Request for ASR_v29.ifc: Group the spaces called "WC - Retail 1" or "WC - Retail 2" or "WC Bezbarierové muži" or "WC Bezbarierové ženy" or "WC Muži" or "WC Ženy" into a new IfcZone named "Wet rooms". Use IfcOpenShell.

First a look at what the model holds.

```python
import ifcopenshell

model = ifcopenshell.open("ASR_v29.ifc")
print(model.schema)
seen = {}
for space in model.by_type("IfcSpace"):
    seen[space.LongName] = seen.get(space.LongName, 0) + 1
for name, count in sorted(seen.items(), key=str):
    print(count, "x", name)
print("zones:", [z.Name for z in model.by_type("IfcZone")][:20])
```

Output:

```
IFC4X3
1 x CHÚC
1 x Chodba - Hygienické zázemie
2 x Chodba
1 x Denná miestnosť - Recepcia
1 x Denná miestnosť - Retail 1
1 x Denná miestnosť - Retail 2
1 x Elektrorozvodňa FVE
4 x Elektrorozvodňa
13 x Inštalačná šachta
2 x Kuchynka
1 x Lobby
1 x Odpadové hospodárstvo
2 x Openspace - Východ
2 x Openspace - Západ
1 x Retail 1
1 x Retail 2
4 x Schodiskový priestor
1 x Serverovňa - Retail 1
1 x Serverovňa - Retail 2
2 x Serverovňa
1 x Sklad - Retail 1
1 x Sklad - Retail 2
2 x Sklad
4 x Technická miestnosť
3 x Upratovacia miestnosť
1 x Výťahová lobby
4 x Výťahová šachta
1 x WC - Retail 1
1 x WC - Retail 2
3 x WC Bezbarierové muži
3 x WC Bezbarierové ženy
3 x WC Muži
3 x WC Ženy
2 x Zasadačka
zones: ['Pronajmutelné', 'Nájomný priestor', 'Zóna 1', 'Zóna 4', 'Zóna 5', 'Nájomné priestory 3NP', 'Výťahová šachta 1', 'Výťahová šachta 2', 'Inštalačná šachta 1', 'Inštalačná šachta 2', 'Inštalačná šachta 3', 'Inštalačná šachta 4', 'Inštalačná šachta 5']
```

```python
import ifcopenshell
import ifcopenshell.api.group
import ifcopenshell.api.root

model = ifcopenshell.open("ASR_v29.ifc")

names = {"WC - Retail 1", "WC - Retail 2", "WC Bezbarierové muži", "WC Bezbarierové ženy", "WC Muži", "WC Ženy"}
spaces = [s for s in model.by_type("IfcSpace") if s.LongName in names]

zone = ifcopenshell.api.root.create_entity(model, ifc_class="IfcZone", name="Wet rooms")
ifcopenshell.api.group.assign_group(model, products=spaces, group=zone)
print(len(spaces), "spaces in", zone.Name)

model.write("ASR_v29_rev.ifc")
```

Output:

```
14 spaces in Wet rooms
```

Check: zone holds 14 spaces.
